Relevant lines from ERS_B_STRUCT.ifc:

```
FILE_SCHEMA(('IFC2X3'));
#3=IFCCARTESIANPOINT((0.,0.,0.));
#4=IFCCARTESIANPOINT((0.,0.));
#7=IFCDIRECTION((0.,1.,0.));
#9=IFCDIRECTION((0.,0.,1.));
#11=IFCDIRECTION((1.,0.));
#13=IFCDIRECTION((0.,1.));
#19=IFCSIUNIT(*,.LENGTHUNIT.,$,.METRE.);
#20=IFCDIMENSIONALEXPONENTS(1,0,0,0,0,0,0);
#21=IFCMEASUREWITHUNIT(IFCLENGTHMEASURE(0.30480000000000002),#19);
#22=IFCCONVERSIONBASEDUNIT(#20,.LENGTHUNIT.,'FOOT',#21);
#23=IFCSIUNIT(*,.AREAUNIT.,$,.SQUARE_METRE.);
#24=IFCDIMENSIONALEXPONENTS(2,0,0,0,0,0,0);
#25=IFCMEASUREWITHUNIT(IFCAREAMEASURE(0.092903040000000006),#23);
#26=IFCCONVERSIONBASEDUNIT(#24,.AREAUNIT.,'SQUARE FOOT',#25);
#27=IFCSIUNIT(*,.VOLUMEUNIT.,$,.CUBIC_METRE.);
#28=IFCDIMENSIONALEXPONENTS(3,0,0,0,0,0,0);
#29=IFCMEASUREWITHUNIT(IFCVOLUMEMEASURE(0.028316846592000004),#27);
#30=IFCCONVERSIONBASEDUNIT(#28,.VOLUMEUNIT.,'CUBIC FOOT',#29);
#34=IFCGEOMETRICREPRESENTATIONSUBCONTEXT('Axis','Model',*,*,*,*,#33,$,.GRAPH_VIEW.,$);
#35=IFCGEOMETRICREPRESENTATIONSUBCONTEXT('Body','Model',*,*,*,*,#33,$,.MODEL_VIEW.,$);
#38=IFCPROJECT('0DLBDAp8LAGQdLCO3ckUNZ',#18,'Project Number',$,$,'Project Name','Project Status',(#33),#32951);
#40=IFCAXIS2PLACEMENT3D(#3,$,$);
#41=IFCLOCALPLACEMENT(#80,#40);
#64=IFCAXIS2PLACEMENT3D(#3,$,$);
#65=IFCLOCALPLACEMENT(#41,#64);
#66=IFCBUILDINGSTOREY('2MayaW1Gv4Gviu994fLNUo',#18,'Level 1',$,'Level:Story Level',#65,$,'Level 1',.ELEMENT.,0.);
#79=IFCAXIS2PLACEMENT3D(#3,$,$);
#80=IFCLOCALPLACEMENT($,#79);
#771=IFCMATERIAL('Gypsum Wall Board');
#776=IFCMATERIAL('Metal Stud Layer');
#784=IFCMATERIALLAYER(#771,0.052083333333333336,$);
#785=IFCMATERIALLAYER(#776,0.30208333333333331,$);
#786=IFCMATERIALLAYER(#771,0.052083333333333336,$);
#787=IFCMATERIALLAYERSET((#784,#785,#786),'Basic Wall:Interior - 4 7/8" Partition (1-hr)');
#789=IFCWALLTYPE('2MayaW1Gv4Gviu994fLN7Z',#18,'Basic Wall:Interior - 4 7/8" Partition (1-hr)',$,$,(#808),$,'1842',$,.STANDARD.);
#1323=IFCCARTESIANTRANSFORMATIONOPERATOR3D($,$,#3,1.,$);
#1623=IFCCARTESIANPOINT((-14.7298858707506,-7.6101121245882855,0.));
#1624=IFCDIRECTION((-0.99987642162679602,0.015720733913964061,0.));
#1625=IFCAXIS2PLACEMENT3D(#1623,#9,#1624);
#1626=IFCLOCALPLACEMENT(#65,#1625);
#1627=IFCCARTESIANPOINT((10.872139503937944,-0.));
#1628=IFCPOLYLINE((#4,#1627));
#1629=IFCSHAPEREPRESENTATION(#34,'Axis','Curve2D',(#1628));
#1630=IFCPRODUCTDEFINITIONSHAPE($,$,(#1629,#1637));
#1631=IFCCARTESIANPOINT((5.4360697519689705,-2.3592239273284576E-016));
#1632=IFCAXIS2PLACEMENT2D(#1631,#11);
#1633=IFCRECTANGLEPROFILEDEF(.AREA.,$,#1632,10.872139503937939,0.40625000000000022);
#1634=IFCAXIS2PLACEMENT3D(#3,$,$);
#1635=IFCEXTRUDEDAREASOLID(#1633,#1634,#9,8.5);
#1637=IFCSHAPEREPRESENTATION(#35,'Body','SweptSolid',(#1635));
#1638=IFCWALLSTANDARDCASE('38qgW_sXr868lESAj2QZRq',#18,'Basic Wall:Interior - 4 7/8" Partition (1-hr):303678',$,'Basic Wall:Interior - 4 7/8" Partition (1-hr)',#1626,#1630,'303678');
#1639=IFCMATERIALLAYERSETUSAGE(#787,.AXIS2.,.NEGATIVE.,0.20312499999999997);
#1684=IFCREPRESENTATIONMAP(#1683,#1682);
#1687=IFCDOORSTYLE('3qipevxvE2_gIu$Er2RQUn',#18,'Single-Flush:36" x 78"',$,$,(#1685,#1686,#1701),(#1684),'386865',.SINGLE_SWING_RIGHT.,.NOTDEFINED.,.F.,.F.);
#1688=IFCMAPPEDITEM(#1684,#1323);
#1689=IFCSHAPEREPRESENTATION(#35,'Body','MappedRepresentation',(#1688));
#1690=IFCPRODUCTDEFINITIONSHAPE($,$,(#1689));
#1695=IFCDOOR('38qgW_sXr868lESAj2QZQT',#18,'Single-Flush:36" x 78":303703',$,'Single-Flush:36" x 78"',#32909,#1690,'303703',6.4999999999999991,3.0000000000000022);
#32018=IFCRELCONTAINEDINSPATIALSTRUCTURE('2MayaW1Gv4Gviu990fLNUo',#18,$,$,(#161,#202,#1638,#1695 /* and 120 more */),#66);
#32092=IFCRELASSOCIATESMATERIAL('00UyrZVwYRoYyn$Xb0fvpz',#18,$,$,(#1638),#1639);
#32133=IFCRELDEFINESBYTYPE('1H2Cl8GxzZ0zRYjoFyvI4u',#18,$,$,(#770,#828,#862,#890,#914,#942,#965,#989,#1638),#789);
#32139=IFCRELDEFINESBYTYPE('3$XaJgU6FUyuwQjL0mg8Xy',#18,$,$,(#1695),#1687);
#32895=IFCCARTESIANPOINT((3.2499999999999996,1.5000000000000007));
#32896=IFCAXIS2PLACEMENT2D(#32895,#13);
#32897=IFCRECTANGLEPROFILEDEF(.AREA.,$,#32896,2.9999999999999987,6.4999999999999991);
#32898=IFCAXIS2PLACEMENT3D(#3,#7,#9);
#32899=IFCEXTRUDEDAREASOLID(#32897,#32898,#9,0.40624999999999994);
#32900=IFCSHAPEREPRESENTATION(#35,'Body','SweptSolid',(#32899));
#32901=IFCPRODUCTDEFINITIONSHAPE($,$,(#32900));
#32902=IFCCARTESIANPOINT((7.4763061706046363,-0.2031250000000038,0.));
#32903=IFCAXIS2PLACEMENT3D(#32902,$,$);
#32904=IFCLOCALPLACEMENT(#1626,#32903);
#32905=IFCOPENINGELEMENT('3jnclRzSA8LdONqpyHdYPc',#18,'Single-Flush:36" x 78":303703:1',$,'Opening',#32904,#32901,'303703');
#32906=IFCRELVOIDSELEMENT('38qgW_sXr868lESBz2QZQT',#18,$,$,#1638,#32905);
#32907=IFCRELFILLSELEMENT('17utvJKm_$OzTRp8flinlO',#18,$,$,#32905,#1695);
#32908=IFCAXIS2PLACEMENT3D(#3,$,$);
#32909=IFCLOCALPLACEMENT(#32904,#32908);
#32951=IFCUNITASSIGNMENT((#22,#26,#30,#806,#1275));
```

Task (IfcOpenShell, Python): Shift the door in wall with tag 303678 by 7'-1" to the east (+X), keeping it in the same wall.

```python
import ifcopenshell
import ifcopenshell.api.geometry
import ifcopenshell.util.placement
import ifcopenshell.util.unit

model = ifcopenshell.open("ERS_B_STRUCT.ifc")
unit_scale = ifcopenshell.util.unit.calculate_unit_scale(model)

door = model.by_id(1695)
opening = door.FillsVoids[0].RelatingOpeningElement
wall = opening.VoidsElements[0].RelatingBuildingElement

wall_matrix = ifcopenshell.util.placement.get_local_placement(wall.ObjectPlacement)
shift = wall_matrix[:3, 0] * -85 * 0.0254 / unit_scale
before = ifcopenshell.util.placement.get_local_placement(door.ObjectPlacement)[:3, 3].copy()

# The door is placed relative to its opening, so it follows when the opening moves.
matrix = ifcopenshell.util.placement.get_local_placement(opening.ObjectPlacement)
matrix[:3, 3] += shift
ifcopenshell.api.geometry.edit_object_placement(
    model, product=opening, matrix=matrix, is_si=False, should_transform_children=True
)

after = ifcopenshell.util.placement.get_local_placement(door.ObjectPlacement)[:3, 3]
print("door moved by", (after - before).round(3) + 0.0)

model.write("ERS_B_STRUCT_edited.ifc")
```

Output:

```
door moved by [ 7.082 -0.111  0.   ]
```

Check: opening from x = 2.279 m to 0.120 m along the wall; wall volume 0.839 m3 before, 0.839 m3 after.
